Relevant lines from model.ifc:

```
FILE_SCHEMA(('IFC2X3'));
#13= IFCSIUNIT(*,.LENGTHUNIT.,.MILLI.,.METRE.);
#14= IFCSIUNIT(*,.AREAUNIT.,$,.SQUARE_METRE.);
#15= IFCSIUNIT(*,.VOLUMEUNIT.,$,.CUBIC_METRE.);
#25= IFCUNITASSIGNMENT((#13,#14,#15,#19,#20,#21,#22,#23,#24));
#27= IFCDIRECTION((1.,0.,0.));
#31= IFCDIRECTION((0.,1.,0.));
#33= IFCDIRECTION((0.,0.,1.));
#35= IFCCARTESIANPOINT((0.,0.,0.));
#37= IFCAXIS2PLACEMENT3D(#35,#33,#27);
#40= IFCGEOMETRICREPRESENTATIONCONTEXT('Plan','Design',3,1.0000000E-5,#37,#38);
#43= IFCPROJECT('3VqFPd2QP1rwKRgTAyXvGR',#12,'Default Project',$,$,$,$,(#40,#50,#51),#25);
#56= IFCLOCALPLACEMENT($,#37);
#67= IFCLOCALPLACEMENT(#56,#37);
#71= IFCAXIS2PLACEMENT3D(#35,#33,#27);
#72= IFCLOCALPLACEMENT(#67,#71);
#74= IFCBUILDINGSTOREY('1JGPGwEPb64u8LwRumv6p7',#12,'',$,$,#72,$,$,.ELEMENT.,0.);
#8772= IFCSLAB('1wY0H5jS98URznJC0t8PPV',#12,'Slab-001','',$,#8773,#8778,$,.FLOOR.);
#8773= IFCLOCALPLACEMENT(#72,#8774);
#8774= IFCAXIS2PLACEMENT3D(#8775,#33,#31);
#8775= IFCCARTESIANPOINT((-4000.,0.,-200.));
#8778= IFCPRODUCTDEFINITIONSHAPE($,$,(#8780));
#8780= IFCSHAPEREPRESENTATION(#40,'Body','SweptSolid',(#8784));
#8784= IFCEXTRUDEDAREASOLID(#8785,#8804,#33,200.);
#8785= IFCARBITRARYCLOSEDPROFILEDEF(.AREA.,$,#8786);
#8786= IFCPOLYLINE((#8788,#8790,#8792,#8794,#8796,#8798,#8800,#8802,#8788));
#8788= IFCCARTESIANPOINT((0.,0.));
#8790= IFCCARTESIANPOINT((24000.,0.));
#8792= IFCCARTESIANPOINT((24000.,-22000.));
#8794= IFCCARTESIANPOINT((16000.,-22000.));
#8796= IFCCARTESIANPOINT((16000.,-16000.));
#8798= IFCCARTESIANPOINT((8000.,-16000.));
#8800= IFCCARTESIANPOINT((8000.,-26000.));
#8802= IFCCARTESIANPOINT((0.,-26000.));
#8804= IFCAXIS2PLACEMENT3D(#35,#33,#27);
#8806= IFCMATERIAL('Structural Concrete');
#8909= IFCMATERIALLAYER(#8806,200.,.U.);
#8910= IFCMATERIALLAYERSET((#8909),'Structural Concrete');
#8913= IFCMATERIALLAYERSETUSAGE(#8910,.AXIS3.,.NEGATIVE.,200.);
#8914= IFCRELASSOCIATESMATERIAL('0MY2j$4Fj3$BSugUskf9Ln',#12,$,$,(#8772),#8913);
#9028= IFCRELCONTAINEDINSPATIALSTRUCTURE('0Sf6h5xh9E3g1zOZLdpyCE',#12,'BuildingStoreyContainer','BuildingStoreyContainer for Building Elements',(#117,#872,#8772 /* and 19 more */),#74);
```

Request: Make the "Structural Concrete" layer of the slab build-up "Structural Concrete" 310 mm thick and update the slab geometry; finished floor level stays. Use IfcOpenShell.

```python
import ifcopenshell
import ifcopenshell.util.element
import ifcopenshell.util.unit

model = ifcopenshell.open("model.ifc")
unit_scale = ifcopenshell.util.unit.calculate_unit_scale(model)

layer_set = model.by_id(8910)
layer = next(l for l in layer_set.MaterialLayers if l.Material and l.Material.Name == "Structural Concrete")
change = 0.31 / unit_scale - layer.LayerThickness
layer.LayerThickness += change

# Geometry does not follow the layer set by itself.
slabs = [e for e in ifcopenshell.util.element.get_elements_by_material(model, layer_set) if e.is_a("IfcSlab")]
for slab in sorted(slabs, key=lambda e: e.id()):
    body = next(r for r in slab.Representation.Representations if r.RepresentationIdentifier == "Body")
    solid = body.Items[0]
    old_depth = solid.Depth
    solid.Depth += change
    # Extruded upwards: lower the start of the extrusion so the top stays.
    x, y, z = solid.Position.Location.Coordinates
    solid.Position.Location = model.createIfcCartesianPoint((x, y, z - change))
    print(slab.id(), f"{old_depth:g} -> {solid.Depth:g}")

model.write("model_rev.ifc")
```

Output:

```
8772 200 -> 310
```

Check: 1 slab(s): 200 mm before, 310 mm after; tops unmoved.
